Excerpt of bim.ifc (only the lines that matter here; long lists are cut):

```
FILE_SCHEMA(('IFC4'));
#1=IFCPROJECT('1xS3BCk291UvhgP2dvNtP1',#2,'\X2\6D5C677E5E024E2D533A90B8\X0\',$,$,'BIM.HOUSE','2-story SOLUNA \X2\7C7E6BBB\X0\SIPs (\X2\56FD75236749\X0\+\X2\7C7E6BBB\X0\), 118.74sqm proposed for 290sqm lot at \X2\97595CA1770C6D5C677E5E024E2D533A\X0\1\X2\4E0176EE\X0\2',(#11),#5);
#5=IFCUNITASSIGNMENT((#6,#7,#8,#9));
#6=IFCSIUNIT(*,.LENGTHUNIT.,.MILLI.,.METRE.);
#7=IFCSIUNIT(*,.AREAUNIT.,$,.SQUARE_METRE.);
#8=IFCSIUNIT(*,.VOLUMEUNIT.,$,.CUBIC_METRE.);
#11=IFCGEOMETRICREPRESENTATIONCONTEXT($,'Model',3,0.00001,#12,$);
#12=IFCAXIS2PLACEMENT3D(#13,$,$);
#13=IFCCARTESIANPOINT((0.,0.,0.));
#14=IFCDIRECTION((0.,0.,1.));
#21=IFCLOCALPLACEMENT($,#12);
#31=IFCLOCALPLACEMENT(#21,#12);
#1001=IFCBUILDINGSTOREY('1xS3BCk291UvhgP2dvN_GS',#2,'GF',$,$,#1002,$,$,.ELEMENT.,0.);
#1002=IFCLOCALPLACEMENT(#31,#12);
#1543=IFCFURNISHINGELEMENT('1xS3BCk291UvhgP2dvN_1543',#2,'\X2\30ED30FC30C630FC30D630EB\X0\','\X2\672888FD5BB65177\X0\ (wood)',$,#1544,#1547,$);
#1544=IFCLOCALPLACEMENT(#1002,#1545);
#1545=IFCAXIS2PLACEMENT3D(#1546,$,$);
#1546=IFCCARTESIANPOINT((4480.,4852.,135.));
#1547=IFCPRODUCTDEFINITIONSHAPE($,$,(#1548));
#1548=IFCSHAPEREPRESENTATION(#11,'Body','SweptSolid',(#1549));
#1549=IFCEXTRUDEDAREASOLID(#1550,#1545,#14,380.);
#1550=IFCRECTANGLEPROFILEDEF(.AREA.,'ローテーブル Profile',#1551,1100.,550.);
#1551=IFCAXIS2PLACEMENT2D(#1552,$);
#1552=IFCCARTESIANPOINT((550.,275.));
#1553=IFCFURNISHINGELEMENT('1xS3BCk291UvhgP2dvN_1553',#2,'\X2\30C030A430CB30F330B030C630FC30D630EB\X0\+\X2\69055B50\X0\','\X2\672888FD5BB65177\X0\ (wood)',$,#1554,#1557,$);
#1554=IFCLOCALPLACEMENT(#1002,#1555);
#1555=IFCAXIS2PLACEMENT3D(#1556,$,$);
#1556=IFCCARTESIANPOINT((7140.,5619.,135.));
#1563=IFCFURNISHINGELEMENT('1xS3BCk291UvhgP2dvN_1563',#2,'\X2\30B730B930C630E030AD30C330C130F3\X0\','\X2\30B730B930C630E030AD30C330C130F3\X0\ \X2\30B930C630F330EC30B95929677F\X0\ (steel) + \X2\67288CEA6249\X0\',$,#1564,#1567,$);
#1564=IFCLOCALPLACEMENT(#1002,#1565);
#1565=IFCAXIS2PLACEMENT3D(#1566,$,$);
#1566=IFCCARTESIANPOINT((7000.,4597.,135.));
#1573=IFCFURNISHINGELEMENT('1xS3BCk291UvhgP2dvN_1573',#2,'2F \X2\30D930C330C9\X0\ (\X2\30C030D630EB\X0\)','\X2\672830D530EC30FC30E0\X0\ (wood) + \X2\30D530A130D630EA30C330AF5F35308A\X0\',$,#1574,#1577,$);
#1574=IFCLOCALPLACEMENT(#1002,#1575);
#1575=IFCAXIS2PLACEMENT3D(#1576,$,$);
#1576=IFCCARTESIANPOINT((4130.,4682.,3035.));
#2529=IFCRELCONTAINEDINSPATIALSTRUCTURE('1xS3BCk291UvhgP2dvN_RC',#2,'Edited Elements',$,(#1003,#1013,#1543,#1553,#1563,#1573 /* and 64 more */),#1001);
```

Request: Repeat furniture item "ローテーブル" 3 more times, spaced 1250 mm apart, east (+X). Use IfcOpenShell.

```python
import numpy as np
import ifcopenshell
import ifcopenshell.api.geometry
import ifcopenshell.api.root
import ifcopenshell.util.element
import ifcopenshell.util.placement
import ifcopenshell.util.unit

model = ifcopenshell.open("bim.ifc")
unit_scale = ifcopenshell.util.unit.calculate_unit_scale(model)


def reuse_history(source, copy):
    """copy_class also copies each property set's owner history, people and application; keep the originals."""
    for rel in copy.IsDefinedBy:
        if rel.is_a("IfcRelDefinesByProperties") and (history := rel.RelatingPropertyDefinition.OwnerHistory):
            rel.RelatingPropertyDefinition.OwnerHistory = source.OwnerHistory
            ifcopenshell.util.element.remove_deep2(model, history)


source = model.by_guid("1xS3BCk291UvhgP2dvN_1543")
base = ifcopenshell.util.placement.get_local_placement(source.ObjectPlacement)
step = np.array([1.0, 0.0, 0.0]) * 1.25 / unit_scale

for i in range(1, 4):
    copy = ifcopenshell.api.root.copy_class(model, product=source)
    copy.Representation = ifcopenshell.util.element.copy_deep(
        model, source.Representation, exclude=["IfcGeometricRepresentationContext", "IfcRepresentationMap"]
    )
    reuse_history(source, copy)
    matrix = base.copy()
    matrix[:3, 3] += i * step
    print("added at", matrix[:3, 3].round(3) + 0.0)
    ifcopenshell.api.geometry.edit_object_placement(model, product=copy, matrix=matrix, is_si=False)

model.write("bim_v2.ifc")
```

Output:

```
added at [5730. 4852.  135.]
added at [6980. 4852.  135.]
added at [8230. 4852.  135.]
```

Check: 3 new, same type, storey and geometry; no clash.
